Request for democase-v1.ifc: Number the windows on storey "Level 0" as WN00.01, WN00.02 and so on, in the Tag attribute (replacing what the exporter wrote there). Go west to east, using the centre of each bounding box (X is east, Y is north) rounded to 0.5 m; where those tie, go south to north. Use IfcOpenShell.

First a look at what the model holds.

```python
import ifcopenshell
import ifcopenshell.util.element
import ifcopenshell.util.placement

model = ifcopenshell.open("democase-v1.ifc")
print(model.schema)
storey = next(s for s in model.by_type("IfcBuildingStorey") if s.Name == "Level 0")
windows = [e for e in ifcopenshell.util.element.get_decomposition(storey) if e.is_a("IfcWindow")]
for e in sorted(windows, key=lambda e: e.id()):
    origin = ifcopenshell.util.placement.get_local_placement(e.ObjectPlacement)[:3, 3]
    print(e.id(), e.Tag, e.Name, origin.round(2) + 0.0, sep=" | ")
```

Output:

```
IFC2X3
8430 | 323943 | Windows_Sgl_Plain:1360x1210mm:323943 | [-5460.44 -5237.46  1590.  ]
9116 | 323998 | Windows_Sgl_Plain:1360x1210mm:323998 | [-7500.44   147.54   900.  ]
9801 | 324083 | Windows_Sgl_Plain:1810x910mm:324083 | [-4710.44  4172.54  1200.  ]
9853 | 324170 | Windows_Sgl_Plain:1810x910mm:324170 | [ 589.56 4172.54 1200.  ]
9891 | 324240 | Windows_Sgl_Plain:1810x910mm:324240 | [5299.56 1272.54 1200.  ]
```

```python
import ifcopenshell
import ifcopenshell.geom
import ifcopenshell.util.element
import ifcopenshell.util.shape

model = ifcopenshell.open("democase-v1.ifc")
settings = ifcopenshell.geom.settings()
settings.set("use-world-coords", True)


def centre(element):
    shape = ifcopenshell.geom.create_shape(settings, element)
    return ifcopenshell.util.shape.get_bbox_centroid(shape.geometry)


storey = next(s for s in model.by_type("IfcBuildingStorey") if s.Name == "Level 0")
windows = [e for e in ifcopenshell.util.element.get_decomposition(storey) if e.is_a("IfcWindow")]

# Insertion points can sit at a corner or the storey origin, so sort by the geometry (in metres).
centres = {e: centre(e) for e in windows}
windows.sort(key=lambda e: (round(centres[e][0] / 0.5), centres[e][1]))

for i, e in enumerate(windows, start=1):
    number = f"WN00.{i:02d}"
    e.Tag = number
    print(e.id(), number)

model.write("democase-v1_updated.ifc")
```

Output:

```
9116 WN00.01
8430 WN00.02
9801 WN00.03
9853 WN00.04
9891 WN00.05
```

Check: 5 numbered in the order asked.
